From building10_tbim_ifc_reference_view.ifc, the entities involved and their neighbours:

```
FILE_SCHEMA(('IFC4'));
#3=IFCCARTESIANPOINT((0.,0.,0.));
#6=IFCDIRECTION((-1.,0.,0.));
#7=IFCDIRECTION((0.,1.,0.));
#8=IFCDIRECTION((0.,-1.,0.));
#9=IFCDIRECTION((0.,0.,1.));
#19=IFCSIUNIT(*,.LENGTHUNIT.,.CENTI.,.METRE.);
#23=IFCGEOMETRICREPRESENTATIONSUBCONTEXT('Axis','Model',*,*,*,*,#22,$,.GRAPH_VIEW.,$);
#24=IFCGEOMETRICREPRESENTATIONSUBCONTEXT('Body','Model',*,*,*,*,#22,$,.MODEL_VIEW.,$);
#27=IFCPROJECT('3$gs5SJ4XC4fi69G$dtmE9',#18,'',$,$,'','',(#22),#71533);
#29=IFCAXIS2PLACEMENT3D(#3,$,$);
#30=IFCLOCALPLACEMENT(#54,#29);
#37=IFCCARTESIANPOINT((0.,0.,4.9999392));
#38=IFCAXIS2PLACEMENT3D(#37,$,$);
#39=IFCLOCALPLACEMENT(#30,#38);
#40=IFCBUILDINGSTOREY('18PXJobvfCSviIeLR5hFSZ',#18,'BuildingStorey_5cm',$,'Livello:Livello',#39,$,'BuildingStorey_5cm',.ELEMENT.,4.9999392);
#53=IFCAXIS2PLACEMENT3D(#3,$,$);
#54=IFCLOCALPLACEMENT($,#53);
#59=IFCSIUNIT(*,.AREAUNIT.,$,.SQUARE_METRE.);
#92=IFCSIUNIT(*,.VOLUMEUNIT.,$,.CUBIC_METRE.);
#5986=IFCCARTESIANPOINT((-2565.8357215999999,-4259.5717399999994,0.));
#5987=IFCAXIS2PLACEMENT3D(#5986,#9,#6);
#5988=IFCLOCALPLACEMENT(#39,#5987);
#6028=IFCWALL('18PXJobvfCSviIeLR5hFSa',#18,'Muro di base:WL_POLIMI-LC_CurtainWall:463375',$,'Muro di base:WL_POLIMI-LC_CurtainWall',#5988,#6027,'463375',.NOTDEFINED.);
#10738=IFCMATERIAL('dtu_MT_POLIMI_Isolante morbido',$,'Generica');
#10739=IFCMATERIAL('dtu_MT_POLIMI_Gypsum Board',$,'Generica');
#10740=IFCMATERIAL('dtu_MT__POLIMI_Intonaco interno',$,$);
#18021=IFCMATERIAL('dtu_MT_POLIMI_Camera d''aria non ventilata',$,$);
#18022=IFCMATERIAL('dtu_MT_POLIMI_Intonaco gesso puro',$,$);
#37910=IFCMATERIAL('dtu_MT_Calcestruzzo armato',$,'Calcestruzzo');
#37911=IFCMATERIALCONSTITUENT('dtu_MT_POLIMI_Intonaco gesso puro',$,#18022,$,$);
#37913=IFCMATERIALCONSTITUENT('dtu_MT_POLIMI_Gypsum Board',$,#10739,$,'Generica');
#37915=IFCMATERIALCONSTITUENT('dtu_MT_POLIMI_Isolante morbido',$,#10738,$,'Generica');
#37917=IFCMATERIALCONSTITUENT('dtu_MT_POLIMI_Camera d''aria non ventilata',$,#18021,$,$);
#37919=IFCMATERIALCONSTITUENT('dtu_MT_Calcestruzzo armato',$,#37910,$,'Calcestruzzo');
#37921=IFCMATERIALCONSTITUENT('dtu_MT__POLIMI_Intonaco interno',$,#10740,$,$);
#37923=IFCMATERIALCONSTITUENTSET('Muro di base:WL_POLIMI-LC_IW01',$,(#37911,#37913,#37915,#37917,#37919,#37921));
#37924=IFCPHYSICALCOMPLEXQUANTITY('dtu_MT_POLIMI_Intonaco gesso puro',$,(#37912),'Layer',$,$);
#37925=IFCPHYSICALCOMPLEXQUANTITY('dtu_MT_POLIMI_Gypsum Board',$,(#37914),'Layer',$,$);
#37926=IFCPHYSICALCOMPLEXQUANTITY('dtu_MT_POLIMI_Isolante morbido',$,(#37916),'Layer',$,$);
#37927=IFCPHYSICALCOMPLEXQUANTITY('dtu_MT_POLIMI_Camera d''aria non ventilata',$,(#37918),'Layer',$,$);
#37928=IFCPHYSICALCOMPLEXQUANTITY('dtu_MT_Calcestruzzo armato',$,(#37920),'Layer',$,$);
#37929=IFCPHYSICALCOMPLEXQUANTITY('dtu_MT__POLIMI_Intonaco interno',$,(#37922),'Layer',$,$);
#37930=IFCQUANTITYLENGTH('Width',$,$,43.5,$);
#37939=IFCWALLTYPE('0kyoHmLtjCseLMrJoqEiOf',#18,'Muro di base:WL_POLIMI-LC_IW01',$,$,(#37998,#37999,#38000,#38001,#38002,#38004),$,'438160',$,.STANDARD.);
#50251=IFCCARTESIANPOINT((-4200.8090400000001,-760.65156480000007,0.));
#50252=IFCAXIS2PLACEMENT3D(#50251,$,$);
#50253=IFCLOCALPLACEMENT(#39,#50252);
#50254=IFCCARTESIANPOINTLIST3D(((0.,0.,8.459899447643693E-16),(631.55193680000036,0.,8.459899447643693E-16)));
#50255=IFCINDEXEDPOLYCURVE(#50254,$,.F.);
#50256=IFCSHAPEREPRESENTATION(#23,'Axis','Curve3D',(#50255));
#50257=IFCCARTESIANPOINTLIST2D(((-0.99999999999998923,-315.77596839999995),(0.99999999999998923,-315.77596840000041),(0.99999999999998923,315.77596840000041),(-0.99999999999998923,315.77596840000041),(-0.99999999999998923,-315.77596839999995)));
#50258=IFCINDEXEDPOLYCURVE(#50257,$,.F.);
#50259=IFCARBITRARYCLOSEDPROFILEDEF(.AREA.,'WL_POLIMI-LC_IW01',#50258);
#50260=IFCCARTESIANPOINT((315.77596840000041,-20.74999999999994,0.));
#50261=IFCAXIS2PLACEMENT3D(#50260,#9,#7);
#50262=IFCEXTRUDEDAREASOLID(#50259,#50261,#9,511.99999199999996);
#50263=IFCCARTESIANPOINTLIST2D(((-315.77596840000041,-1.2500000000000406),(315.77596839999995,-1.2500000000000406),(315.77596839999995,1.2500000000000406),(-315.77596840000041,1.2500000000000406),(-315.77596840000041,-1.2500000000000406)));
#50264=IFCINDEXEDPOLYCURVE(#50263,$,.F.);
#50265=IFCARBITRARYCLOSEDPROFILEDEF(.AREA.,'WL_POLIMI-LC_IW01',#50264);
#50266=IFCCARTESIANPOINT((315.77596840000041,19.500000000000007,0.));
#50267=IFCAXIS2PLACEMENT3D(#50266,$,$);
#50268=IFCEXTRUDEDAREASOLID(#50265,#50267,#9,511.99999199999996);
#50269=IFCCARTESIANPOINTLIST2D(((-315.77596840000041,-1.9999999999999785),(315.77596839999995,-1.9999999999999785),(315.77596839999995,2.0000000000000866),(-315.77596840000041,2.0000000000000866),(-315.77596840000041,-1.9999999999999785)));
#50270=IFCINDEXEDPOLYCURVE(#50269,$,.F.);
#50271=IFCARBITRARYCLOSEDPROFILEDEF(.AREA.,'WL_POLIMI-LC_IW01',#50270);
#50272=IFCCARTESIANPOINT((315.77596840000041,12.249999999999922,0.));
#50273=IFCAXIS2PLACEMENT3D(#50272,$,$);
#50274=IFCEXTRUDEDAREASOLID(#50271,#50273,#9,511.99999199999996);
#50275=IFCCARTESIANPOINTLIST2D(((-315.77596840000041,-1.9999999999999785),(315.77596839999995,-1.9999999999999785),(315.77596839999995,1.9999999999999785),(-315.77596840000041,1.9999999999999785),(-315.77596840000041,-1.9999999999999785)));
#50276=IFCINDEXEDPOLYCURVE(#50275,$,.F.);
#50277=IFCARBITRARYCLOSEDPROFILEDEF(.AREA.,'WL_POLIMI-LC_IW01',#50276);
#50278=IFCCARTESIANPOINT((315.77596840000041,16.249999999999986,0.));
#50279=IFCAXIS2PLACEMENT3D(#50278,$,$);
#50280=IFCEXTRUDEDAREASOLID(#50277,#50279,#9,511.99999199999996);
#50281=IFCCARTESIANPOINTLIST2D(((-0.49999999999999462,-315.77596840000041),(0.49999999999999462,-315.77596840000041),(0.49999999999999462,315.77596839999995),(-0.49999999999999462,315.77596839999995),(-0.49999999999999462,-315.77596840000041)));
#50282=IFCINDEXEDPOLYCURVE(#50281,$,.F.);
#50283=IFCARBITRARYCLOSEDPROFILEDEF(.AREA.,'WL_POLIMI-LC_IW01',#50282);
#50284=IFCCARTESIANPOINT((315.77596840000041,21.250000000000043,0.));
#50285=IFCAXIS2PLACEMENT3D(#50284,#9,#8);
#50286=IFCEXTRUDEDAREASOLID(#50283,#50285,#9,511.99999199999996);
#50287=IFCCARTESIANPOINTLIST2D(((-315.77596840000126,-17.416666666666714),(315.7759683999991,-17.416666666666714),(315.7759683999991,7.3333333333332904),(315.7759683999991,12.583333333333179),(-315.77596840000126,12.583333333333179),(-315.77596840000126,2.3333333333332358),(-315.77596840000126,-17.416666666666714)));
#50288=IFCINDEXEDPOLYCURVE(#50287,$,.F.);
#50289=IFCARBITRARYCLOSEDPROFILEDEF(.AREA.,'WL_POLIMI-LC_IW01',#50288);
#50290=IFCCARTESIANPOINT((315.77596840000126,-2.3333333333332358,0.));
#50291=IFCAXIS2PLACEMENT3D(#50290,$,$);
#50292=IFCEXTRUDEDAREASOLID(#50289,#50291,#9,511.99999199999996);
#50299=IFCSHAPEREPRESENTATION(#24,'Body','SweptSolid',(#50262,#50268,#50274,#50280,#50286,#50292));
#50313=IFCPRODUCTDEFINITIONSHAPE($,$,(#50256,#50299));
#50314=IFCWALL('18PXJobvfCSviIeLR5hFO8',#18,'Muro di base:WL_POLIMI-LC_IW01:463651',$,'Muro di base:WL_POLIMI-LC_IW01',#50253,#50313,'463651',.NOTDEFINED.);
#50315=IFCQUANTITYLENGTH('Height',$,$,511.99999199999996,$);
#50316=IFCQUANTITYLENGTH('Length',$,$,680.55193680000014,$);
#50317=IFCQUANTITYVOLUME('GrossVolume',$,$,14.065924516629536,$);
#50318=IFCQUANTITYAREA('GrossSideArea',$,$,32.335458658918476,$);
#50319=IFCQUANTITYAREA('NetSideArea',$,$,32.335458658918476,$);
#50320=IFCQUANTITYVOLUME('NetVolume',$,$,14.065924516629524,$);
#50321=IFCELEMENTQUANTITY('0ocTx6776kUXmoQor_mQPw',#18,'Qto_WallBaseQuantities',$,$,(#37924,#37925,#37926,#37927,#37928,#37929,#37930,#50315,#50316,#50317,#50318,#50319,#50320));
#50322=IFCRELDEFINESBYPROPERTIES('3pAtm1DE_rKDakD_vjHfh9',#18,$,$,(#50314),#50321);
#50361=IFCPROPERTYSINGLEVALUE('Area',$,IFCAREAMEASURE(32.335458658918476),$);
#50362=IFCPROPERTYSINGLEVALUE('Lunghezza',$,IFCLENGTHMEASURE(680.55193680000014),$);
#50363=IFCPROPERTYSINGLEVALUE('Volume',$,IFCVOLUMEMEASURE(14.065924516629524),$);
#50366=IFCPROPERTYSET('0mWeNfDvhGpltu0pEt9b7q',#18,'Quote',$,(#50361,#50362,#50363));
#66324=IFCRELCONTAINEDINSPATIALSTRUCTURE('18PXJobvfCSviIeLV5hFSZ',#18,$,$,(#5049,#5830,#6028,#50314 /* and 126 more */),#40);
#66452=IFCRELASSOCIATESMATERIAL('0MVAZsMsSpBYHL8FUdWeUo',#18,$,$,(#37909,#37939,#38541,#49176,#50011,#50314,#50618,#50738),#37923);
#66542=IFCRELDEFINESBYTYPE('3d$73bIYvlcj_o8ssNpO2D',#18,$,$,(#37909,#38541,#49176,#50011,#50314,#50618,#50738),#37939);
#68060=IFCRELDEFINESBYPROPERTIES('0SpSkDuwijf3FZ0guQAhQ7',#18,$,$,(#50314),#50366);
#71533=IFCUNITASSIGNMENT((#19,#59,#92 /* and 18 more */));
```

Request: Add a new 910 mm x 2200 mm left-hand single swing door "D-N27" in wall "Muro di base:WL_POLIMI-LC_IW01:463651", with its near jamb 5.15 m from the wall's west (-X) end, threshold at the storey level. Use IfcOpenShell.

```python
import numpy as np
import ifcopenshell
import ifcopenshell.api.feature
import ifcopenshell.api.geometry
import ifcopenshell.api.pset
import ifcopenshell.api.root
import ifcopenshell.api.spatial
import ifcopenshell.geom
import ifcopenshell.util.element
import ifcopenshell.util.placement
import ifcopenshell.util.representation
import ifcopenshell.util.shape
import ifcopenshell.util.unit

model = ifcopenshell.open("building10_tbim_ifc_reference_view.ifc")
unit_scale = ifcopenshell.util.unit.calculate_unit_scale(model)
area_scale = ifcopenshell.util.unit.calculate_unit_scale(model, "AREAUNIT")
volume_scale = ifcopenshell.util.unit.calculate_unit_scale(model, "VOLUMEUNIT")
settings = ifcopenshell.geom.settings()


def volume(element):
    """Net volume in cubic metres, openings subtracted."""
    shape = ifcopenshell.geom.create_shape(settings, element)
    return ifcopenshell.util.shape.get_volume(shape.geometry)


wall = model.by_guid("18PXJobvfCSviIeLR5hFO8")
storey = ifcopenshell.util.element.get_container(wall, ifc_class="IfcBuildingStorey")
context = ifcopenshell.util.representation.get_context(model, "Model", "Body", "MODEL_VIEW")
before = volume(wall)

width, height, from_end, sill = 0.91, 2.2, 5.15, 0.0  # metres

# The wall runs along its own X axis, and the end named is its -X end.
wall_shape = ifcopenshell.geom.create_shape(settings, wall)
x, y, z = ifcopenshell.util.shape.get_vertices(wall_shape.geometry).T
start = x.min() + from_end
face, thickness = float(y.min()), float(y.max() - y.min())
wall_matrix = ifcopenshell.util.placement.get_local_placement(wall.ObjectPlacement)
level = ifcopenshell.util.placement.get_local_placement(storey.ObjectPlacement)[2, 3]


def in_wall(x, y):
    """Placement at x, y metres in the wall's axes, at sill height."""
    matrix = wall_matrix.copy()
    matrix[:, 3] = wall_matrix @ np.array([x / unit_scale, y / unit_scale, 0.0, 1.0])
    matrix[2, 3] = level + sill / unit_scale
    return matrix


# Opening: a box that overshoots both wall faces by 50 mm.
opening = ifcopenshell.api.root.create_entity(model, ifc_class="IfcOpeningElement", predefined_type="OPENING")
box = ifcopenshell.api.geometry.add_wall_representation(
    model, context=context, length=width, height=height, thickness=thickness + 0.1
)
ifcopenshell.api.geometry.assign_representation(model, product=opening, representation=box)
ifcopenshell.api.geometry.edit_object_placement(model, product=opening, matrix=in_wall(start, face - 0.05), is_si=False)
ifcopenshell.api.feature.add_feature(model, feature=opening, element=wall)

door = ifcopenshell.api.root.create_entity(model, ifc_class="IfcDoor", name="D-N27", predefined_type="DOOR")
door.OverallWidth, door.OverallHeight = width / unit_scale, height / unit_scale
door.OperationType = "SINGLE_SWING_LEFT"
body = ifcopenshell.api.geometry.add_door_representation(
    model,
    context=context,
    overall_width=door.OverallWidth,
    overall_height=door.OverallHeight,
    operation_type="SINGLE_SWING_LEFT",
    lining_properties={"LiningDepth": thickness / unit_scale, "ThresholdDepth": thickness / unit_scale},
)
ifcopenshell.api.geometry.assign_representation(model, product=door, representation=body)
ifcopenshell.api.spatial.assign_container(model, products=[door], relating_structure=storey)
ifcopenshell.api.feature.add_filling(model, opening=opening, element=door)

# The lining spans the wall, so the door starts at the wall face.
ifcopenshell.api.geometry.edit_object_placement(model, product=door, matrix=in_wall(start, face), is_si=False)

after = volume(wall)

# Update the wall's stored quantities.
qto = model.by_id(ifcopenshell.util.element.get_pset(wall, "Qto_WallBaseQuantities", should_inherit=False)["id"])
ifcopenshell.api.pset.edit_qto(model, qto=qto, properties={
    "NetSideArea": after / thickness / area_scale,
    "NetVolume": after / volume_scale,
})
pset = model.by_id(ifcopenshell.util.element.get_pset(wall, "Quote", should_inherit=False)["id"])
ifcopenshell.api.pset.edit_pset(model, pset=pset, properties={
    "Area": model.create_entity("IfcAreaMeasure", after / thickness / area_scale),
    "Volume": model.create_entity("IfcVolumeMeasure", after / volume_scale),
})

print(f"wall volume {before:.3f} -> {after:.3f} m3")

model.write("building10_tbim_ifc_reference_view_v2.ifc")
```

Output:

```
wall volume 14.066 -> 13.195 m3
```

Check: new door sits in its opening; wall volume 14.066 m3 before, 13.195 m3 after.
